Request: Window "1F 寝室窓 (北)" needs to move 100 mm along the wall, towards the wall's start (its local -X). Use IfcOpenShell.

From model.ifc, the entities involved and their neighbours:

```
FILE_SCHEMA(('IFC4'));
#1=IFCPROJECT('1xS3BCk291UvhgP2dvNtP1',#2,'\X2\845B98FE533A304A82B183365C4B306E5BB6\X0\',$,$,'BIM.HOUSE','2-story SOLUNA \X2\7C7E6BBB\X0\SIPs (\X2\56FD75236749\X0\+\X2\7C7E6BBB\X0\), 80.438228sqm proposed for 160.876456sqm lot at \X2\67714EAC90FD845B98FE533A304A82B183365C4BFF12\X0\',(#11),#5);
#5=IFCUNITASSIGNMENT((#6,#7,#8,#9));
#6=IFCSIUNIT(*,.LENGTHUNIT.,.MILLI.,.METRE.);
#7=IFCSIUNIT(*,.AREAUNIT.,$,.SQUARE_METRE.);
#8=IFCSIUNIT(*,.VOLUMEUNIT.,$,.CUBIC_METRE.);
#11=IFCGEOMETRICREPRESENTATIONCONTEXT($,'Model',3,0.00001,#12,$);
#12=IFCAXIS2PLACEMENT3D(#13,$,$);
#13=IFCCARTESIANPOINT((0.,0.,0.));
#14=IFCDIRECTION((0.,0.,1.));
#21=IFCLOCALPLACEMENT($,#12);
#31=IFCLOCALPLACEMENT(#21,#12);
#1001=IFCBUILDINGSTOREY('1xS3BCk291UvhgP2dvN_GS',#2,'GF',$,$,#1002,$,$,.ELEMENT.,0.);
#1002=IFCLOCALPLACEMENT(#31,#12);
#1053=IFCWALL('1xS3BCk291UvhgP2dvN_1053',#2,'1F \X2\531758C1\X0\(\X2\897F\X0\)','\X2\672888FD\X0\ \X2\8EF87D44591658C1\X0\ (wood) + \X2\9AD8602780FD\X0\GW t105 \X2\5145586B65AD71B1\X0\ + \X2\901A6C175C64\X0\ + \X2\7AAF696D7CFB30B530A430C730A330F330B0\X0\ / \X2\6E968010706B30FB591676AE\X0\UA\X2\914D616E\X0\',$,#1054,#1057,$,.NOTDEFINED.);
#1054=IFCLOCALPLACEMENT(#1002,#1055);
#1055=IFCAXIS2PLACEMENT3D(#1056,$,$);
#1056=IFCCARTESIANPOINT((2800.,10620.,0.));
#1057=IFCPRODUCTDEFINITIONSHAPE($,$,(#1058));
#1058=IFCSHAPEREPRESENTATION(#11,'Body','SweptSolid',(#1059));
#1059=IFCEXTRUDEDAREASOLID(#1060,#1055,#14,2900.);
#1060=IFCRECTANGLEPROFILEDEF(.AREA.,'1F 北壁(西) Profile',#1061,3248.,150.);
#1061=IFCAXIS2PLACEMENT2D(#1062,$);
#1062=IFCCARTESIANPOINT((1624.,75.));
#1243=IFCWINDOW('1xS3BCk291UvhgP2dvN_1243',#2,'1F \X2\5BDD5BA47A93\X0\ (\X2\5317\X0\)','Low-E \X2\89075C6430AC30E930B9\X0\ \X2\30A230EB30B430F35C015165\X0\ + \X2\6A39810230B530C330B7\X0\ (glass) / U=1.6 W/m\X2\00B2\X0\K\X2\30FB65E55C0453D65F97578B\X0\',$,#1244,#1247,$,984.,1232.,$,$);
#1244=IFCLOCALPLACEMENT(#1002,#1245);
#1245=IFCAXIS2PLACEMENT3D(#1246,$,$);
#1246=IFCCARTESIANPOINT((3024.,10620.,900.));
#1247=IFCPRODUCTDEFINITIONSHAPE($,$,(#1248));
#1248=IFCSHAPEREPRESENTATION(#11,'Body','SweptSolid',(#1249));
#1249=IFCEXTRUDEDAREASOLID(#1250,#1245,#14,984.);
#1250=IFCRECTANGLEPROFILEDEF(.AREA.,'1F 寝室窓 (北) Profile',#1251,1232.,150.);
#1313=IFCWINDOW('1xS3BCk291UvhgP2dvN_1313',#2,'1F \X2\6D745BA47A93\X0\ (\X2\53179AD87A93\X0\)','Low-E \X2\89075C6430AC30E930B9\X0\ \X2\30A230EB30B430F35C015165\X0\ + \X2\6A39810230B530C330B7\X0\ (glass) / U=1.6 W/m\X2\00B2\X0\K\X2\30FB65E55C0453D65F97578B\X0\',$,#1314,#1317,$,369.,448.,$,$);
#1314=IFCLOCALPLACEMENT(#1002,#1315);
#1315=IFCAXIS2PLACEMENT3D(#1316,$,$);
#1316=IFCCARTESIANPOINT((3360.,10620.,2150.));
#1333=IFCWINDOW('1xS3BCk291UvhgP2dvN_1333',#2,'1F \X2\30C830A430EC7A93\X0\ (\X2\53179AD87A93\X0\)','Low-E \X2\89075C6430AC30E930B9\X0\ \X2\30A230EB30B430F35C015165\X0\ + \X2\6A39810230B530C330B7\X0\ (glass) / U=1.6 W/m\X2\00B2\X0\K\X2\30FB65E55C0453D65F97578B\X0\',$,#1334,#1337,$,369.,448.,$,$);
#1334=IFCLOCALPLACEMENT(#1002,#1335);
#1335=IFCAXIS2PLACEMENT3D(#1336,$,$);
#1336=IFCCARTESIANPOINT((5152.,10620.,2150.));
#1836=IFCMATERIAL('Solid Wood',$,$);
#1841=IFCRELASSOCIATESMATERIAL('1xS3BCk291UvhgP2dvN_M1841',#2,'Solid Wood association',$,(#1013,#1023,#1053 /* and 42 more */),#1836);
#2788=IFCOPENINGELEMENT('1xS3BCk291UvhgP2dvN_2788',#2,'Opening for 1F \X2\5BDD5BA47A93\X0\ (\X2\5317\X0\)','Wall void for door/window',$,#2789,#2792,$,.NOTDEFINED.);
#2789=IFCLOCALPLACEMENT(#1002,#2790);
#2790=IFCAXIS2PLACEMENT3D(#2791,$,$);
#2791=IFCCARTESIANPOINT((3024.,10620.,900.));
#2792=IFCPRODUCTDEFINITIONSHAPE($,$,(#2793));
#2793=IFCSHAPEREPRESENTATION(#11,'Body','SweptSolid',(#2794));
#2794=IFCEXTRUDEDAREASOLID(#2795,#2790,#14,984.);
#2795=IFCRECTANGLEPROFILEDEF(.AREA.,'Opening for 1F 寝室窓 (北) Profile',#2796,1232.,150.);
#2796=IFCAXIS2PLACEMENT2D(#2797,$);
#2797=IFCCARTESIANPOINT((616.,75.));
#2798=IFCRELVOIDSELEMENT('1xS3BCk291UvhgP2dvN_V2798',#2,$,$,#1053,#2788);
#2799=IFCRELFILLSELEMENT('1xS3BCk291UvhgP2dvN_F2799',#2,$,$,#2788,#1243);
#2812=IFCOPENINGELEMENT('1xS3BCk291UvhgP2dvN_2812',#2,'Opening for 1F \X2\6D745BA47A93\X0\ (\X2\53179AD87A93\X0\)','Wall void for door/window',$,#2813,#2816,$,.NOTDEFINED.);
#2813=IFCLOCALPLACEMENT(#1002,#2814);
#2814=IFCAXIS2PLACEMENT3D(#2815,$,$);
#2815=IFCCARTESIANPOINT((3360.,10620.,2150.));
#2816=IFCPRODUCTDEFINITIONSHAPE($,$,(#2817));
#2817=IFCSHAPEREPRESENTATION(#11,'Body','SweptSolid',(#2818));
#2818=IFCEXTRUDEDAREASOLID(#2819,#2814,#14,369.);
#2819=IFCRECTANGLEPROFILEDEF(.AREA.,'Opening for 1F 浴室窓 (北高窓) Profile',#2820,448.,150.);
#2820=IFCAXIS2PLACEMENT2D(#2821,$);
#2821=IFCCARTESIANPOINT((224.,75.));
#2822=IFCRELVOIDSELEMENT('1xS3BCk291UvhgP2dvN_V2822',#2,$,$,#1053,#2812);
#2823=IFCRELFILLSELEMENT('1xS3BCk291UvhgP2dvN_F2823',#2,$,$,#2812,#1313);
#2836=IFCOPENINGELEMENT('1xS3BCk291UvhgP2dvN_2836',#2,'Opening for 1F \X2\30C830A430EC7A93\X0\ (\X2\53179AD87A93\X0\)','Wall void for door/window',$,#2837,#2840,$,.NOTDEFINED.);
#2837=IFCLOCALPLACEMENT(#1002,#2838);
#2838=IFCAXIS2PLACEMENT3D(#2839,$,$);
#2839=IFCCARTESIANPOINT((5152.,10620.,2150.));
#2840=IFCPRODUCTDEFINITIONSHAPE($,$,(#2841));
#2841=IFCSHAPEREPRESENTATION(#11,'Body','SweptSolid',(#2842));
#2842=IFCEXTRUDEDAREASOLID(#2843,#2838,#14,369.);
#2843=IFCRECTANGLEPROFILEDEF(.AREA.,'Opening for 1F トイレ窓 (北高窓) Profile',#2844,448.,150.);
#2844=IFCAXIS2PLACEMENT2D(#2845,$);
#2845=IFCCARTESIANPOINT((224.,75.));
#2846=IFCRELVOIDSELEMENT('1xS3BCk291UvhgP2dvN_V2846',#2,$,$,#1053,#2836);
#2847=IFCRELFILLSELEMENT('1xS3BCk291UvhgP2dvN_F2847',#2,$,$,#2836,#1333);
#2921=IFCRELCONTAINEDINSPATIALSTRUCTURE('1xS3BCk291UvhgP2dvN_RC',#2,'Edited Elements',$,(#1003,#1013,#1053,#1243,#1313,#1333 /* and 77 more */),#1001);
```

```python
import ifcopenshell
import ifcopenshell.api.geometry
import ifcopenshell.util.placement

model = ifcopenshell.open("model.ifc")

window = model.by_guid("1xS3BCk291UvhgP2dvN_1243")
opening = window.FillsVoids[0].RelatingOpeningElement
wall = opening.VoidsElements[0].RelatingBuildingElement

wall_matrix = ifcopenshell.util.placement.get_local_placement(wall.ObjectPlacement)
shift = wall_matrix[:3, 0] * -100.0
before = ifcopenshell.util.placement.get_local_placement(window.ObjectPlacement)[:3, 3].copy()

# The window is not placed relative to its opening, so move both.
for product in (opening, window):
    matrix = ifcopenshell.util.placement.get_local_placement(product.ObjectPlacement)
    matrix[:3, 3] += shift
    ifcopenshell.api.geometry.edit_object_placement(model, product=product, matrix=matrix, is_si=False)

after = ifcopenshell.util.placement.get_local_placement(window.ObjectPlacement)[:3, 3]
print("window moved by", (after - before).round(3) + 0.0)

model.write("model-out.ifc")
```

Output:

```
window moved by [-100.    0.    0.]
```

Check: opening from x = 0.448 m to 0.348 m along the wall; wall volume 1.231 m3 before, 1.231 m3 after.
